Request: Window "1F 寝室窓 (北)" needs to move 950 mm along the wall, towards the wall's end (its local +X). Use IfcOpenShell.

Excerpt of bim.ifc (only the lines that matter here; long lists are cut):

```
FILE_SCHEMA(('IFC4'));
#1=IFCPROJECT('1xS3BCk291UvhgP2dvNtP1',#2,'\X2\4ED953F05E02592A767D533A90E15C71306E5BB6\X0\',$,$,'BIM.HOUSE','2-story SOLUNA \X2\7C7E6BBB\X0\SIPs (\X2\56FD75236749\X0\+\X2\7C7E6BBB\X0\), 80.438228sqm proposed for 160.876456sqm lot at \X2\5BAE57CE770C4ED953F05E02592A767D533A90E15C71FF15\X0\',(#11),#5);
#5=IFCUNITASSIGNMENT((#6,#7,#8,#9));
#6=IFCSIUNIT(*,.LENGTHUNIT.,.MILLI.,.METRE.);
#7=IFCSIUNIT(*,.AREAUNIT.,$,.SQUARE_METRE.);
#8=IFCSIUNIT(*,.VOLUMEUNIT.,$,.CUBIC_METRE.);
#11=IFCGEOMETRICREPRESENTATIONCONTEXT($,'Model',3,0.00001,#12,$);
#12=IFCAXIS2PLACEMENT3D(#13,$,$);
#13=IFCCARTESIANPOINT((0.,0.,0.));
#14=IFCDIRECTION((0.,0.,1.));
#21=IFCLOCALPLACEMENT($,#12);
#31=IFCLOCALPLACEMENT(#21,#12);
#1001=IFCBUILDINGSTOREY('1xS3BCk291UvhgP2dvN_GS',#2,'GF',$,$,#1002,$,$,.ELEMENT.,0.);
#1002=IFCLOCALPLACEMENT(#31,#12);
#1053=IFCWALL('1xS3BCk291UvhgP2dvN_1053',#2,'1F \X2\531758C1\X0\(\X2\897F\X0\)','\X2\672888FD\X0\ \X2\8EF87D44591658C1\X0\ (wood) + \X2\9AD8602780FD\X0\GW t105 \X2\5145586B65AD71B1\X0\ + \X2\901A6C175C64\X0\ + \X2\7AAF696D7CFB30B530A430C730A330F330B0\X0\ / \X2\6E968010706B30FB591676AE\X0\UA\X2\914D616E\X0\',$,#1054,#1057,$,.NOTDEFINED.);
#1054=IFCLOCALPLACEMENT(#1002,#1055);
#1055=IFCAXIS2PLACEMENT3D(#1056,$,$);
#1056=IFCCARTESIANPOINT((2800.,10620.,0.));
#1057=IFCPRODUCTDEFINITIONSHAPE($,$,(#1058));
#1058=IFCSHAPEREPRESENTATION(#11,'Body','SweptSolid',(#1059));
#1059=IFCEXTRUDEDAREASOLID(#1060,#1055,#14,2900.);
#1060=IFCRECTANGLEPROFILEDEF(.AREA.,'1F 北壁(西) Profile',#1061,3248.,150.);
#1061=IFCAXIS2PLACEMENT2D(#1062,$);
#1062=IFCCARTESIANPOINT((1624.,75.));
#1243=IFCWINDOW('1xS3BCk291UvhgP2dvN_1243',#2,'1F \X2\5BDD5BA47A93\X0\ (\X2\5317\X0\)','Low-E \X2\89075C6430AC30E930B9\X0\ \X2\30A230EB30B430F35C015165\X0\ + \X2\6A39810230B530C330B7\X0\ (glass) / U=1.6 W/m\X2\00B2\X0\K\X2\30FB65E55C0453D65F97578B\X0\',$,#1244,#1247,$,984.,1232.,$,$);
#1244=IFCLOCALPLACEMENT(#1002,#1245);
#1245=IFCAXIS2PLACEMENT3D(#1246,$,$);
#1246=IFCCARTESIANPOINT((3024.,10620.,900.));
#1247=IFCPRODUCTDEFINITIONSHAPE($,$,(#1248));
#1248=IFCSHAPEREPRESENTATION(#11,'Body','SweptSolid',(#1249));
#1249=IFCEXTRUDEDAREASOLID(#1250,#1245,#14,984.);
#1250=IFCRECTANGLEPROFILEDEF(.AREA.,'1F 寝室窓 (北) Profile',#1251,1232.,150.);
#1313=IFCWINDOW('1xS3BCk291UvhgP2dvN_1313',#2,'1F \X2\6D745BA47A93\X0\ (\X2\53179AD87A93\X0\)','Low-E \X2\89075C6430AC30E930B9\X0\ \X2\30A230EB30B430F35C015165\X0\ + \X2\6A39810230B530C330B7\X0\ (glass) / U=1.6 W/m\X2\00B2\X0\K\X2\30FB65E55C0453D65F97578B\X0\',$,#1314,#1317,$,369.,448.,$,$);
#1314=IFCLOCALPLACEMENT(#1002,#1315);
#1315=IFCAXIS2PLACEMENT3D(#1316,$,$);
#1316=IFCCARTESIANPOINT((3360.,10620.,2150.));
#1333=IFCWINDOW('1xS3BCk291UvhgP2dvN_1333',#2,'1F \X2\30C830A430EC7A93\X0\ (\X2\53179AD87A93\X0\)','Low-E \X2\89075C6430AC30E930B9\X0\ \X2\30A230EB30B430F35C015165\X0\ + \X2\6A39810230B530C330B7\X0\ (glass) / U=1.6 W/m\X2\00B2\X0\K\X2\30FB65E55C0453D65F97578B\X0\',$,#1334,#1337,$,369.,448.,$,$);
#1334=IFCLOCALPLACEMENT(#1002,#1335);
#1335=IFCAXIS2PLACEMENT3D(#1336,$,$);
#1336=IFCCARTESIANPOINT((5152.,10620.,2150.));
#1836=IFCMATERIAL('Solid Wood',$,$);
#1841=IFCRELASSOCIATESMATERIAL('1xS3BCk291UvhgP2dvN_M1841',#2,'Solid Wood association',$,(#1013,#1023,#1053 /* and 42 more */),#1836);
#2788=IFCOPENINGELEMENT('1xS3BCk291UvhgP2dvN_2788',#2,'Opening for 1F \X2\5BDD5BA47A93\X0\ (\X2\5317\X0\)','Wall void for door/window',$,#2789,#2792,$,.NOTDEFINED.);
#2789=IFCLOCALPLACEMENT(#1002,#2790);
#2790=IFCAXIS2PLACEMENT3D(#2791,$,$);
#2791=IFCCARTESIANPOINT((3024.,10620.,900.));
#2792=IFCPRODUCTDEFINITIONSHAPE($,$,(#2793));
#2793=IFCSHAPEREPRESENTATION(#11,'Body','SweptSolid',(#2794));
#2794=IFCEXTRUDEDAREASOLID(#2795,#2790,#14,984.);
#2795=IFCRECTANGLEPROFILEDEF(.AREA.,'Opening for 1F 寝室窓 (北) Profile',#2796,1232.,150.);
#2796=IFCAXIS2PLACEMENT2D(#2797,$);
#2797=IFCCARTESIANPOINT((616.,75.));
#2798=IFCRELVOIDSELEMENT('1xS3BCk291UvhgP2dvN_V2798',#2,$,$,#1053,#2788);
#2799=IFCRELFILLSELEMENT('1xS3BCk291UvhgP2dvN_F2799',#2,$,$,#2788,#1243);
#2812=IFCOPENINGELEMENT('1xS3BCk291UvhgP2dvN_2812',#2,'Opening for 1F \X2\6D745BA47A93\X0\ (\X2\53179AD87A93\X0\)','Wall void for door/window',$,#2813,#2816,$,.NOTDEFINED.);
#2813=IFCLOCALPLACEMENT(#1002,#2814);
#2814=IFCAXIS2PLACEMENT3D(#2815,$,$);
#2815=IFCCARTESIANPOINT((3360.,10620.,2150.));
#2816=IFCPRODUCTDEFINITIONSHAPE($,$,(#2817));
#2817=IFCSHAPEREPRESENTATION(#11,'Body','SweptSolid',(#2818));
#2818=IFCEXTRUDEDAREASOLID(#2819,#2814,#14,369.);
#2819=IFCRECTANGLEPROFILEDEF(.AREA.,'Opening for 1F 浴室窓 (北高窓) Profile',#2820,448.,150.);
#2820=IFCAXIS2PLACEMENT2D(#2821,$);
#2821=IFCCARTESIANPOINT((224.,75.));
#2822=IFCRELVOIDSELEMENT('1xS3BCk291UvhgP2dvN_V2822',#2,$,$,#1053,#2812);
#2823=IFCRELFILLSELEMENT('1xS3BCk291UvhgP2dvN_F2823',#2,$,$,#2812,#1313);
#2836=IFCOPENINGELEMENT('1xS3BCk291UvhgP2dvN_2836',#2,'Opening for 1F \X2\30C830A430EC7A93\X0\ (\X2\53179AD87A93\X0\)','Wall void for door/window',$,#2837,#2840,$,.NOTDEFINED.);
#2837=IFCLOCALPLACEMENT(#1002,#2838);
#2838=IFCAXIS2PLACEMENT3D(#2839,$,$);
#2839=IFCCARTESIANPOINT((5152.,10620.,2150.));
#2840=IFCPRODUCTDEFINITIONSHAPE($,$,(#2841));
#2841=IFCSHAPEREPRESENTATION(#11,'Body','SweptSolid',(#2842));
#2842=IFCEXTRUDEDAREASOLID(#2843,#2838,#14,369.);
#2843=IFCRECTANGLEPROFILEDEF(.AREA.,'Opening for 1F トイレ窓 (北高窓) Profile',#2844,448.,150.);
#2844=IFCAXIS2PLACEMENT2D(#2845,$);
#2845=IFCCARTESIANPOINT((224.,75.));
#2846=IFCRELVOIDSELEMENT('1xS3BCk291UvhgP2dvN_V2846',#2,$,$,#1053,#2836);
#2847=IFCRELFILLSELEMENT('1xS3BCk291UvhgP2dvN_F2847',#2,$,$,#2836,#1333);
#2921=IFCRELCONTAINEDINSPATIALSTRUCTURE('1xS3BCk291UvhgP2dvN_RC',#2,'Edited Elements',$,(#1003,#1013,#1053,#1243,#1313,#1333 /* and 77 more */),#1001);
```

```python
import ifcopenshell
import ifcopenshell.api.geometry
import ifcopenshell.util.placement
import ifcopenshell.util.unit

model = ifcopenshell.open("bim.ifc")
unit_scale = ifcopenshell.util.unit.calculate_unit_scale(model)

window = model.by_guid("1xS3BCk291UvhgP2dvN_1243")
opening = window.FillsVoids[0].RelatingOpeningElement
wall = opening.VoidsElements[0].RelatingBuildingElement

wall_matrix = ifcopenshell.util.placement.get_local_placement(wall.ObjectPlacement)
shift = wall_matrix[:3, 0] * 0.95 / unit_scale
before = ifcopenshell.util.placement.get_local_placement(window.ObjectPlacement)[:3, 3].copy()

# The window is not placed relative to its opening, so move both.
for product in (opening, window):
    matrix = ifcopenshell.util.placement.get_local_placement(product.ObjectPlacement)
    matrix[:3, 3] += shift
    ifcopenshell.api.geometry.edit_object_placement(model, product=product, matrix=matrix, is_si=False)

after = ifcopenshell.util.placement.get_local_placement(window.ObjectPlacement)[:3, 3]
print("window moved by", (after - before).round(3) + 0.0)

model.write("bim_updated.ifc")
```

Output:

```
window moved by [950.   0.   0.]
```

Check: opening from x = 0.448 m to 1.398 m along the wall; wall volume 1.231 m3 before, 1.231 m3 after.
